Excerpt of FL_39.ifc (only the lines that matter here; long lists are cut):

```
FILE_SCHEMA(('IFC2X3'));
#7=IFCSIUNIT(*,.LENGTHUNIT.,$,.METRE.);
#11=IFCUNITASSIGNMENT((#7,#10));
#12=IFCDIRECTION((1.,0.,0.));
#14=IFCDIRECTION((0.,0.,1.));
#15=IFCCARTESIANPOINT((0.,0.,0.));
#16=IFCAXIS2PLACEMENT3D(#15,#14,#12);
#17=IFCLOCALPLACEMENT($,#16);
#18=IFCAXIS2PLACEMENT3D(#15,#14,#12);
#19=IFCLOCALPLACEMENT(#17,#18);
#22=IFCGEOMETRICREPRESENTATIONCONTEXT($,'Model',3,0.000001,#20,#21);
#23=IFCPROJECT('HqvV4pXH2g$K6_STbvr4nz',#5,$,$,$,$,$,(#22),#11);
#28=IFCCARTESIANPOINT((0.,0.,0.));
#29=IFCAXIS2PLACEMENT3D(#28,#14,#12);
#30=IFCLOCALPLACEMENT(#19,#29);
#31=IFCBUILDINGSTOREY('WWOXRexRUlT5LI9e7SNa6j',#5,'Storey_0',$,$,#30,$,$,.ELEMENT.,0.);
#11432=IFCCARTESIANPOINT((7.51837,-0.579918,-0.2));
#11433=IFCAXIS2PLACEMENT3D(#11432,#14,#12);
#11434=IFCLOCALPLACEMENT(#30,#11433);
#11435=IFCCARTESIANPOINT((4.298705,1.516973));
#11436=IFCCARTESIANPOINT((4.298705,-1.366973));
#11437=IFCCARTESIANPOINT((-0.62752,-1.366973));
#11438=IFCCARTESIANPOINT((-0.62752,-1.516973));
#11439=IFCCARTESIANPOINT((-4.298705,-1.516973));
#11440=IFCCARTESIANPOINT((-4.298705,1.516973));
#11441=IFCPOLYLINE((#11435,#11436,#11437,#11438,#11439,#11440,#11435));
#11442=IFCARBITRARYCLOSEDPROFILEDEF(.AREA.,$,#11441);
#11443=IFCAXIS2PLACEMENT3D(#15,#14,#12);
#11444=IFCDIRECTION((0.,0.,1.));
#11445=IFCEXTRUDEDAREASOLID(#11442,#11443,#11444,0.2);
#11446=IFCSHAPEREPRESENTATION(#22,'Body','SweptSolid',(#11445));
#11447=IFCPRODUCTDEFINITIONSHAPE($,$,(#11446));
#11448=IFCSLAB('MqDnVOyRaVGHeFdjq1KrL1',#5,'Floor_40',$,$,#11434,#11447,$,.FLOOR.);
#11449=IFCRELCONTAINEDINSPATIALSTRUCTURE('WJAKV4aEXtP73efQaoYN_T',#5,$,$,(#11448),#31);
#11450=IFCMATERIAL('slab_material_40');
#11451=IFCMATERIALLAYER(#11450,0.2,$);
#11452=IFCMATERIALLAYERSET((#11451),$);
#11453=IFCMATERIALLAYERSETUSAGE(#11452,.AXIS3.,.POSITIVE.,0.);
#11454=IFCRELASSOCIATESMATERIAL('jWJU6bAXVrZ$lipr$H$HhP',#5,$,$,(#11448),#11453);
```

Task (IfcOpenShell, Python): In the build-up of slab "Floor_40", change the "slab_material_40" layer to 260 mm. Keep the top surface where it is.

```python
import ifcopenshell
import ifcopenshell.util.element
import ifcopenshell.util.unit

model = ifcopenshell.open("FL_39.ifc")
unit_scale = ifcopenshell.util.unit.calculate_unit_scale(model)

layer_set = model.by_id(11452)
layer = next(l for l in layer_set.MaterialLayers if l.Material and l.Material.Name == "slab_material_40")
change = 0.26 / unit_scale - layer.LayerThickness
layer.LayerThickness += change

# Geometry does not follow the layer set by itself.
slabs = [e for e in ifcopenshell.util.element.get_elements_by_material(model, layer_set) if e.is_a("IfcSlab")]
for slab in sorted(slabs, key=lambda e: e.id()):
    body = next(r for r in slab.Representation.Representations if r.RepresentationIdentifier == "Body")
    solid = body.Items[0]
    old_depth = solid.Depth
    solid.Depth += change
    # Extruded upwards: lower the start of the extrusion so the top stays.
    x, y, z = solid.Position.Location.Coordinates
    solid.Position.Location = model.createIfcCartesianPoint((x, y, z - change))
    print(slab.id(), f"{old_depth:g} -> {solid.Depth:g}")

# The layers are counted up from the underside, which has moved.
for usage in {ifcopenshell.util.element.get_material(slab) for slab in slabs}:
    usage.OffsetFromReferenceLine -= change

model.write("FL_39_rev.ifc")
```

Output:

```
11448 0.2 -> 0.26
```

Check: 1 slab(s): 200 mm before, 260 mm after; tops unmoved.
